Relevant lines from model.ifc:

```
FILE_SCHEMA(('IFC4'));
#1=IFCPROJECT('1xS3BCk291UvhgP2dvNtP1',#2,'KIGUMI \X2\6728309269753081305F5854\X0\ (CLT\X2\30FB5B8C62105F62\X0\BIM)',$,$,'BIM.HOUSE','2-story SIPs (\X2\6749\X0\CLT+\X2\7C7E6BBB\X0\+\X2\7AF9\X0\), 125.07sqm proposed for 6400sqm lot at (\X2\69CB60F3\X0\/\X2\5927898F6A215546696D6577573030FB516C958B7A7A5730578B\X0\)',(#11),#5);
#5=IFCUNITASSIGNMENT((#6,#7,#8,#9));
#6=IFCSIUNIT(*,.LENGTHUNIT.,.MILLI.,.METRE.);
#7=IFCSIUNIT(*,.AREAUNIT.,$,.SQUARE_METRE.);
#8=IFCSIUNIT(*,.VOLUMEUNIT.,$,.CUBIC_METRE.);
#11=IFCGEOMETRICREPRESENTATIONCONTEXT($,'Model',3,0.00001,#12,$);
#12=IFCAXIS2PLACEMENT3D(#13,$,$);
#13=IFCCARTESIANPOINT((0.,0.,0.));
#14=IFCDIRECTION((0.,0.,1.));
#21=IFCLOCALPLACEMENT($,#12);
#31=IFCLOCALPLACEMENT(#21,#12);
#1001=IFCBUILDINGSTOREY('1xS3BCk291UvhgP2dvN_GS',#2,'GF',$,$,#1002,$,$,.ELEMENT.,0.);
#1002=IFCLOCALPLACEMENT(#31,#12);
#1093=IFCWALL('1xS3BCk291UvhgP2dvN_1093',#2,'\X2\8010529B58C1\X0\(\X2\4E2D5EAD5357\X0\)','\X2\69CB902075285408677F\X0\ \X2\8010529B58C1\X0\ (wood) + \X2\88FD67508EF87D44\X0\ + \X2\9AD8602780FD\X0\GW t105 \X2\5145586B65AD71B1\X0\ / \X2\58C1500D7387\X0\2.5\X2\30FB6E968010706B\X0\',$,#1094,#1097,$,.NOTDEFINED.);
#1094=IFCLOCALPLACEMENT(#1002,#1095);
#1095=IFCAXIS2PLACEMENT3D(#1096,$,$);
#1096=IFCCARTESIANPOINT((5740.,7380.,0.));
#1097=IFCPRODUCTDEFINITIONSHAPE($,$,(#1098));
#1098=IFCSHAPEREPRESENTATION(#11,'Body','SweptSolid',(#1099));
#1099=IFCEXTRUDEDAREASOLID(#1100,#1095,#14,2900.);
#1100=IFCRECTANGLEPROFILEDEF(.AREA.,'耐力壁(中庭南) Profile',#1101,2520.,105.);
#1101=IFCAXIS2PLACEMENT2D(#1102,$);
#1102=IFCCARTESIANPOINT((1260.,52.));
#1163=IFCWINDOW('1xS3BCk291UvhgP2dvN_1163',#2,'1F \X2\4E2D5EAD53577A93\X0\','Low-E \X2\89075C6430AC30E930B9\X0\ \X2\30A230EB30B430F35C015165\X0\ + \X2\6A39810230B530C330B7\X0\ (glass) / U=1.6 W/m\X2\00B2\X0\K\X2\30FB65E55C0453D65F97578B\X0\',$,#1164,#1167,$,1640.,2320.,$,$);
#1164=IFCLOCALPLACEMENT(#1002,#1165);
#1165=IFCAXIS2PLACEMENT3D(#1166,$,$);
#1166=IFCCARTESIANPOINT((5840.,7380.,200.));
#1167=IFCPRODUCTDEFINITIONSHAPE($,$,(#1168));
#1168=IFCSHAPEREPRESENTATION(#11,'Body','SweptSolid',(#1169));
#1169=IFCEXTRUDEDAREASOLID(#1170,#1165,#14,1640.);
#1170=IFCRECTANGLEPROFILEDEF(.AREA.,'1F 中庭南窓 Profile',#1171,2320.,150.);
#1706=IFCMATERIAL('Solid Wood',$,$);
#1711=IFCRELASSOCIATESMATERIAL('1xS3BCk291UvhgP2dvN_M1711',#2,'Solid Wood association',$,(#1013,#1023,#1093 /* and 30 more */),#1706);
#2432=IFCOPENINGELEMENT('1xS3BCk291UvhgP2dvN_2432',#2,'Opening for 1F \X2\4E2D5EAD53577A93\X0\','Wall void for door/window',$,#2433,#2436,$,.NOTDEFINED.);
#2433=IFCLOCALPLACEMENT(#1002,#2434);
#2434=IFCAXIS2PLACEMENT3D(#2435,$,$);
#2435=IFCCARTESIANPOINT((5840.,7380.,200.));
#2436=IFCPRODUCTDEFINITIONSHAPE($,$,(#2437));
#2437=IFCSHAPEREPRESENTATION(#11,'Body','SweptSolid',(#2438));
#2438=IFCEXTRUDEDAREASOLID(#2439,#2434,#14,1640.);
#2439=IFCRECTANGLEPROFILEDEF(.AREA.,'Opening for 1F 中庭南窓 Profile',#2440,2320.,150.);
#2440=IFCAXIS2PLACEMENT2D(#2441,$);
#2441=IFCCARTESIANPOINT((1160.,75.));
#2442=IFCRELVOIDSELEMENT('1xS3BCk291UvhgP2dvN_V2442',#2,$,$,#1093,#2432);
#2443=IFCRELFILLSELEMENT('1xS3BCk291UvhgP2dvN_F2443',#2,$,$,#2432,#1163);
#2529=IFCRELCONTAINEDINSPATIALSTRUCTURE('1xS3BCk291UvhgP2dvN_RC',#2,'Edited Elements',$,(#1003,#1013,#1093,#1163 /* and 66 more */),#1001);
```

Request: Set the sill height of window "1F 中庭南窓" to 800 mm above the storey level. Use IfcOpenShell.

```python
import numpy as np
import ifcopenshell
import ifcopenshell.api.geometry
import ifcopenshell.geom
import ifcopenshell.util.element
import ifcopenshell.util.placement
import ifcopenshell.util.shape
import ifcopenshell.util.unit

model = ifcopenshell.open("model.ifc")
unit_scale = ifcopenshell.util.unit.calculate_unit_scale(model)

window = model.by_guid("1xS3BCk291UvhgP2dvN_1163")
opening = window.FillsVoids[0].RelatingOpeningElement
storey = ifcopenshell.util.element.get_container(window, ifc_class="IfcBuildingStorey")
level = ifcopenshell.util.placement.get_local_placement(storey.ObjectPlacement)[2, 3]

# The opening's origin need not be at the sill, so measure its lowest point.
shape = ifcopenshell.geom.create_shape(ifcopenshell.geom.settings(), opening)
bottom = ifcopenshell.util.shape.get_shape_bottom_elevation(shape, shape.geometry) / unit_scale
dz = level + 0.8 / unit_scale - bottom

shift = np.array([0.0, 0.0, dz])
# The window is not placed relative to its opening, so move both.
for product in (opening, window):
    matrix = ifcopenshell.util.placement.get_local_placement(product.ObjectPlacement)
    matrix[:3, 3] += shift
    ifcopenshell.api.geometry.edit_object_placement(model, product=product, matrix=matrix, is_si=False)

print(f"moved by {dz * unit_scale:+.3f} m")

model.write("model_rev.ifc")
```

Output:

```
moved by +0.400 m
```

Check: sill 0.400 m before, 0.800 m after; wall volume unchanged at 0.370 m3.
